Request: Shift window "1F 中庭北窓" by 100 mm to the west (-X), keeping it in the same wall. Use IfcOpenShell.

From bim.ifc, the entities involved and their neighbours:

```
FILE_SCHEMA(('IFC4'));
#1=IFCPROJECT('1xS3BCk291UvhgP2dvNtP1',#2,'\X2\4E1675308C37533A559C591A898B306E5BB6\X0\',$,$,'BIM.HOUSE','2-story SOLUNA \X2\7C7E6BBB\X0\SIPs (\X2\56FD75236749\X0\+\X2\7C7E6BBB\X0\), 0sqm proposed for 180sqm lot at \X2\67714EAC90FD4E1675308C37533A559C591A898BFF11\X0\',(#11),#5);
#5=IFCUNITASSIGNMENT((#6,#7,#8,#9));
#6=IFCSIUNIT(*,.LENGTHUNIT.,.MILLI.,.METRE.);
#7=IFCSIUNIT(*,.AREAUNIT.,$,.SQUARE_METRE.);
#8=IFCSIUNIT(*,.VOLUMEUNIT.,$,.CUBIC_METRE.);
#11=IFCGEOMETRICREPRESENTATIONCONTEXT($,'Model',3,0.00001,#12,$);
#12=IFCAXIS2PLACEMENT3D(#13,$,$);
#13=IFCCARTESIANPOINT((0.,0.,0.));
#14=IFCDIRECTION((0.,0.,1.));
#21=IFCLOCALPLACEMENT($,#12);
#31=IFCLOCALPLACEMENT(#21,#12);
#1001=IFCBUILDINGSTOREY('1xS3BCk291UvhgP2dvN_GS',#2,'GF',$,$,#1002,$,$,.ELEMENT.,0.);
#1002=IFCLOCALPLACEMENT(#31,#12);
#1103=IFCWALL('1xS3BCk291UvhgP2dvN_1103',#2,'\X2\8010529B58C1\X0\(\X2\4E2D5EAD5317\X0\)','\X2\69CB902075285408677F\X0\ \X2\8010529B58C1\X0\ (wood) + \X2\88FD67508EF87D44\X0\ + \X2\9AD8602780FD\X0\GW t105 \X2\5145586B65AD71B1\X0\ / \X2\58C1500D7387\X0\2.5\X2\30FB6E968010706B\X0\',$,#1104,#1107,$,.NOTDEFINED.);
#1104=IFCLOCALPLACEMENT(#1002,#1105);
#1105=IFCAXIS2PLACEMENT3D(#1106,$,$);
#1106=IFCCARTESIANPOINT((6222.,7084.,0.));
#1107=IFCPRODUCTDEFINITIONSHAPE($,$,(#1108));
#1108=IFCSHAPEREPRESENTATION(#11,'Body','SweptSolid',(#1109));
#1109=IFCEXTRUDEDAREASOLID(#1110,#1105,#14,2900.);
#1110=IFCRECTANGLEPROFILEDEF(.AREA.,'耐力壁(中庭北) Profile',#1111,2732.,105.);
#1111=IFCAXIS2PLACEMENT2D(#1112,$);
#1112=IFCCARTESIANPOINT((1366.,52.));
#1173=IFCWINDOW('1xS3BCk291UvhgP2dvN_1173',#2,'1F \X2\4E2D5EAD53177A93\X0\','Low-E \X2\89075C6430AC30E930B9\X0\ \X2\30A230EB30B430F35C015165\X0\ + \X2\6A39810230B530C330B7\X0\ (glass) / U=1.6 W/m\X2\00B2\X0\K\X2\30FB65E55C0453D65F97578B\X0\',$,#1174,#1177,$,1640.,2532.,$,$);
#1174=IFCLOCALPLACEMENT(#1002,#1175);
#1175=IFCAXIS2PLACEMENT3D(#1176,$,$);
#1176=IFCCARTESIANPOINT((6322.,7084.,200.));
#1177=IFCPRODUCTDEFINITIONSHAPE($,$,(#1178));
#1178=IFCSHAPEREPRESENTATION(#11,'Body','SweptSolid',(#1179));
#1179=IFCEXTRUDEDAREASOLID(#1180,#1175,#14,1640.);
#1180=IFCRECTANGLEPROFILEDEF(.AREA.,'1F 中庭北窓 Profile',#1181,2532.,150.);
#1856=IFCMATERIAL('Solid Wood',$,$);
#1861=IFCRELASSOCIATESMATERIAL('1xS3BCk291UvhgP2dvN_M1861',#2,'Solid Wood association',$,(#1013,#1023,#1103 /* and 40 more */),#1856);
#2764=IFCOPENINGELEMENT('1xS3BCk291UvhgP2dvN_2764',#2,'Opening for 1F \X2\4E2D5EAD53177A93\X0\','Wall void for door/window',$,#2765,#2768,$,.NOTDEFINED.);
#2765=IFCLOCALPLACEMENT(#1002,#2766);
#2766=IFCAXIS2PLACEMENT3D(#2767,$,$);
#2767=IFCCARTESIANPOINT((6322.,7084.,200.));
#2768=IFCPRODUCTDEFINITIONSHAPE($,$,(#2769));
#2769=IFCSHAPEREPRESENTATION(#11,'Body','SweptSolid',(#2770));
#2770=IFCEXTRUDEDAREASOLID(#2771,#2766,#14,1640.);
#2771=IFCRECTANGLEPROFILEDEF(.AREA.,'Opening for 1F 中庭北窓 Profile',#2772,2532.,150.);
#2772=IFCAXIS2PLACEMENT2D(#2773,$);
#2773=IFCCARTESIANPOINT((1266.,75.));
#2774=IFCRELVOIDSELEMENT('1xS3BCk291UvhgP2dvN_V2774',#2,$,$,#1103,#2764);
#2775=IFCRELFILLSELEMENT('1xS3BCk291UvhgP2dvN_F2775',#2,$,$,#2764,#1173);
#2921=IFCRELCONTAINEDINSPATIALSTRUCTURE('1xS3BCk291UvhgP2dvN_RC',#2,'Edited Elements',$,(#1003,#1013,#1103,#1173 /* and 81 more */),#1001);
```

```python
import ifcopenshell
import ifcopenshell.api.geometry
import ifcopenshell.util.placement

model = ifcopenshell.open("bim.ifc")

window = model.by_guid("1xS3BCk291UvhgP2dvN_1173")
opening = window.FillsVoids[0].RelatingOpeningElement
wall = opening.VoidsElements[0].RelatingBuildingElement

wall_matrix = ifcopenshell.util.placement.get_local_placement(wall.ObjectPlacement)
shift = wall_matrix[:3, 0] * -100.0
before = ifcopenshell.util.placement.get_local_placement(window.ObjectPlacement)[:3, 3].copy()

# The window is not placed relative to its opening, so move both.
for product in (opening, window):
    matrix = ifcopenshell.util.placement.get_local_placement(product.ObjectPlacement)
    matrix[:3, 3] += shift
    ifcopenshell.api.geometry.edit_object_placement(model, product=product, matrix=matrix, is_si=False)

after = ifcopenshell.util.placement.get_local_placement(window.ObjectPlacement)[:3, 3]
print("window moved by", (after - before).round(3) + 0.0)

model.write("bim_edited.ifc")
```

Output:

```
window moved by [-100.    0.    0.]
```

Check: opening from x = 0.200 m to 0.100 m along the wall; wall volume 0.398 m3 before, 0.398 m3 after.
